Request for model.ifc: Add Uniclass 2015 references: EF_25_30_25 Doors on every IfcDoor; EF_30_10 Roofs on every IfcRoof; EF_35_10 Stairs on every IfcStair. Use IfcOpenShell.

First a look at what the model holds.

```python
import ifcopenshell

model = ifcopenshell.open("model.ifc")
print(model.schema)
print("classifications:", [c.Name for c in model.by_type("IfcClassification")])
for ifc_class in ("IfcDoor", "IfcRoof", "IfcStair", "IfcWall", "IfcWindow"):
    print(ifc_class, len(model.by_type(ifc_class)))
```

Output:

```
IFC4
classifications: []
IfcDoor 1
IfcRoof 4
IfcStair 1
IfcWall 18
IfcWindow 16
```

```python
import ifcopenshell
import ifcopenshell.api.classification

model = ifcopenshell.open("model.ifc")

system = ifcopenshell.api.classification.add_classification(model, classification="Uniclass 2015")

codes = {
    "IfcDoor": ("EF_25_30_25", "Doors"),
    "IfcRoof": ("EF_30_10", "Roofs"),
    "IfcStair": ("EF_35_10", "Stairs"),
}
for ifc_class, (code, name) in codes.items():
    products = model.by_type(ifc_class)
    ifcopenshell.api.classification.add_reference(
        model, products=products, classification=system, identification=code, name=name
    )
    print(code, len(products))

model.write("model_updated.ifc")
```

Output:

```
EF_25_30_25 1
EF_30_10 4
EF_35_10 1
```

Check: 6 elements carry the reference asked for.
